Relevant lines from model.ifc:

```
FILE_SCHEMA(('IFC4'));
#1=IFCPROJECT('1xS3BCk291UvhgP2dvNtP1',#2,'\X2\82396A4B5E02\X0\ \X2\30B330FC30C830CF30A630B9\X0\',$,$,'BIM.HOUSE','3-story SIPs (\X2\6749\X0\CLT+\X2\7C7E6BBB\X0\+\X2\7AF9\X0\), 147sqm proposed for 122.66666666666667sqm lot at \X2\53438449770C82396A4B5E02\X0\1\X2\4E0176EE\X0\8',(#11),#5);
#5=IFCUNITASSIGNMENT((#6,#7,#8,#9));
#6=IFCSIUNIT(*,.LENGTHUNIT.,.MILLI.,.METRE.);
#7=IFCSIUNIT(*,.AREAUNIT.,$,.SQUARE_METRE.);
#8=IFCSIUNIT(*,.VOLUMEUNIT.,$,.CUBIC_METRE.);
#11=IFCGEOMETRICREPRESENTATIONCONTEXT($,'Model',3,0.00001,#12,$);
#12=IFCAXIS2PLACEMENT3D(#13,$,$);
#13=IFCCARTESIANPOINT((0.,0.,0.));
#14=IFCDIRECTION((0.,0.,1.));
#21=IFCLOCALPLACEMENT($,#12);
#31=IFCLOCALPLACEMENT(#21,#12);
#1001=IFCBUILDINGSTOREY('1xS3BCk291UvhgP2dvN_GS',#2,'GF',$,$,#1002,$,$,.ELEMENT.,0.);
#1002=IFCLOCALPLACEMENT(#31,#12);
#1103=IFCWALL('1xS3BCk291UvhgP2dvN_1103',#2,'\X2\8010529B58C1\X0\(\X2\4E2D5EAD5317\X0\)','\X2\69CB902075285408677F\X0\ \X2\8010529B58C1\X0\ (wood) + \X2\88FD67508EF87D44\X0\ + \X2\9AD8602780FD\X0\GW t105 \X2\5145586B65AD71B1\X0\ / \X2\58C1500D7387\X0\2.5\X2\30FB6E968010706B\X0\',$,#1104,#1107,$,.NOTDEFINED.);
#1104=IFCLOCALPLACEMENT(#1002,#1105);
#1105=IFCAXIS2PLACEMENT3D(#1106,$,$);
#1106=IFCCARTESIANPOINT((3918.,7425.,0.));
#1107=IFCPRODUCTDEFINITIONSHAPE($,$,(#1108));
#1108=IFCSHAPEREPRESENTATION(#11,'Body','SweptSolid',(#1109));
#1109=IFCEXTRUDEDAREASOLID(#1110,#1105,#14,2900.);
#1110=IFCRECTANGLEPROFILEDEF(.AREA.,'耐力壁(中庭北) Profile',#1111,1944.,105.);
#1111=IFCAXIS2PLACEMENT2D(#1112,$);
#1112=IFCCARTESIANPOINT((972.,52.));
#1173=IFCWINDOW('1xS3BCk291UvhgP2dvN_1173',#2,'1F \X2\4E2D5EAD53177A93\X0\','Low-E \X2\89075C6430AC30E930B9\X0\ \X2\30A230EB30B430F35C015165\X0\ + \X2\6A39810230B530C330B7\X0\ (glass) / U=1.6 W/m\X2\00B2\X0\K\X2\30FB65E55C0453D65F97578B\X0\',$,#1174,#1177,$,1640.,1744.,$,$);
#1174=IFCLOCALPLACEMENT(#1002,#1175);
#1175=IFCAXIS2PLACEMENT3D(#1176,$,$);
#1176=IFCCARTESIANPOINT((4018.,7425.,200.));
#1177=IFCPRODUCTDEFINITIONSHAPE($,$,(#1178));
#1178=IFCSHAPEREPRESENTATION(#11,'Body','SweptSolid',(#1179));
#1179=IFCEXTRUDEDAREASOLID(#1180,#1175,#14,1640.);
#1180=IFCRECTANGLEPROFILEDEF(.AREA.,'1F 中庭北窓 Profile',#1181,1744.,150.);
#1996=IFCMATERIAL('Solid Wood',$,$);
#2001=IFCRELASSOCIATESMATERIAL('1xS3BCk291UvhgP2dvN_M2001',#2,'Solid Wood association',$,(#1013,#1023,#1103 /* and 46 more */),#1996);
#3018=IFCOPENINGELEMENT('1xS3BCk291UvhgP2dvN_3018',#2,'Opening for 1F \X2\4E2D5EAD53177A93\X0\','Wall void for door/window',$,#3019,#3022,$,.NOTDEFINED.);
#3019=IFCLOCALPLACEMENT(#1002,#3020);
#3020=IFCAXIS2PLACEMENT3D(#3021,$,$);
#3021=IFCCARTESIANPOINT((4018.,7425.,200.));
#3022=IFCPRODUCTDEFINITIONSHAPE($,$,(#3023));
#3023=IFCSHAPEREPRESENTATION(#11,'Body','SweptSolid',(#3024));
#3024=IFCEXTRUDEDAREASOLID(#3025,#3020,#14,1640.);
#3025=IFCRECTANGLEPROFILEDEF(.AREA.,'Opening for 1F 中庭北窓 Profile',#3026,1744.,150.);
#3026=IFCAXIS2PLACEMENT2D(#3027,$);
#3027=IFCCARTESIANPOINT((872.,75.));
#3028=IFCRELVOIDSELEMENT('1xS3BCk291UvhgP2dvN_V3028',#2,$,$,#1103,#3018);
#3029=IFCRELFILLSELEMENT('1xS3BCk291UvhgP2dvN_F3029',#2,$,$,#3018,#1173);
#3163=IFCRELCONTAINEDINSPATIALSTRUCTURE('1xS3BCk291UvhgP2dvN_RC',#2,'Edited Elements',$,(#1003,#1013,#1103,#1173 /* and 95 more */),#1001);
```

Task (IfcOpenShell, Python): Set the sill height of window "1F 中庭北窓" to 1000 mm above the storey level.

```python
import numpy as np
import ifcopenshell
import ifcopenshell.api.geometry
import ifcopenshell.geom
import ifcopenshell.util.element
import ifcopenshell.util.placement
import ifcopenshell.util.shape
import ifcopenshell.util.unit

model = ifcopenshell.open("model.ifc")
unit_scale = ifcopenshell.util.unit.calculate_unit_scale(model)

window = model.by_guid("1xS3BCk291UvhgP2dvN_1173")
opening = window.FillsVoids[0].RelatingOpeningElement
storey = ifcopenshell.util.element.get_container(window, ifc_class="IfcBuildingStorey")
level = ifcopenshell.util.placement.get_local_placement(storey.ObjectPlacement)[2, 3]

# The opening's origin need not be at the sill, so measure its lowest point.
shape = ifcopenshell.geom.create_shape(ifcopenshell.geom.settings(), opening)
bottom = ifcopenshell.util.shape.get_shape_bottom_elevation(shape, shape.geometry) / unit_scale
dz = level + 1 / unit_scale - bottom

shift = np.array([0.0, 0.0, dz])
# The window is not placed relative to its opening, so move both.
for product in (opening, window):
    matrix = ifcopenshell.util.placement.get_local_placement(product.ObjectPlacement)
    matrix[:3, 3] += shift
    ifcopenshell.api.geometry.edit_object_placement(model, product=product, matrix=matrix, is_si=False)

print(f"moved by {dz * unit_scale:+.3f} m")

model.write("model_rev.ifc")
```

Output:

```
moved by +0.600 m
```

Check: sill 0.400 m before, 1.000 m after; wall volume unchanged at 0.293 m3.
